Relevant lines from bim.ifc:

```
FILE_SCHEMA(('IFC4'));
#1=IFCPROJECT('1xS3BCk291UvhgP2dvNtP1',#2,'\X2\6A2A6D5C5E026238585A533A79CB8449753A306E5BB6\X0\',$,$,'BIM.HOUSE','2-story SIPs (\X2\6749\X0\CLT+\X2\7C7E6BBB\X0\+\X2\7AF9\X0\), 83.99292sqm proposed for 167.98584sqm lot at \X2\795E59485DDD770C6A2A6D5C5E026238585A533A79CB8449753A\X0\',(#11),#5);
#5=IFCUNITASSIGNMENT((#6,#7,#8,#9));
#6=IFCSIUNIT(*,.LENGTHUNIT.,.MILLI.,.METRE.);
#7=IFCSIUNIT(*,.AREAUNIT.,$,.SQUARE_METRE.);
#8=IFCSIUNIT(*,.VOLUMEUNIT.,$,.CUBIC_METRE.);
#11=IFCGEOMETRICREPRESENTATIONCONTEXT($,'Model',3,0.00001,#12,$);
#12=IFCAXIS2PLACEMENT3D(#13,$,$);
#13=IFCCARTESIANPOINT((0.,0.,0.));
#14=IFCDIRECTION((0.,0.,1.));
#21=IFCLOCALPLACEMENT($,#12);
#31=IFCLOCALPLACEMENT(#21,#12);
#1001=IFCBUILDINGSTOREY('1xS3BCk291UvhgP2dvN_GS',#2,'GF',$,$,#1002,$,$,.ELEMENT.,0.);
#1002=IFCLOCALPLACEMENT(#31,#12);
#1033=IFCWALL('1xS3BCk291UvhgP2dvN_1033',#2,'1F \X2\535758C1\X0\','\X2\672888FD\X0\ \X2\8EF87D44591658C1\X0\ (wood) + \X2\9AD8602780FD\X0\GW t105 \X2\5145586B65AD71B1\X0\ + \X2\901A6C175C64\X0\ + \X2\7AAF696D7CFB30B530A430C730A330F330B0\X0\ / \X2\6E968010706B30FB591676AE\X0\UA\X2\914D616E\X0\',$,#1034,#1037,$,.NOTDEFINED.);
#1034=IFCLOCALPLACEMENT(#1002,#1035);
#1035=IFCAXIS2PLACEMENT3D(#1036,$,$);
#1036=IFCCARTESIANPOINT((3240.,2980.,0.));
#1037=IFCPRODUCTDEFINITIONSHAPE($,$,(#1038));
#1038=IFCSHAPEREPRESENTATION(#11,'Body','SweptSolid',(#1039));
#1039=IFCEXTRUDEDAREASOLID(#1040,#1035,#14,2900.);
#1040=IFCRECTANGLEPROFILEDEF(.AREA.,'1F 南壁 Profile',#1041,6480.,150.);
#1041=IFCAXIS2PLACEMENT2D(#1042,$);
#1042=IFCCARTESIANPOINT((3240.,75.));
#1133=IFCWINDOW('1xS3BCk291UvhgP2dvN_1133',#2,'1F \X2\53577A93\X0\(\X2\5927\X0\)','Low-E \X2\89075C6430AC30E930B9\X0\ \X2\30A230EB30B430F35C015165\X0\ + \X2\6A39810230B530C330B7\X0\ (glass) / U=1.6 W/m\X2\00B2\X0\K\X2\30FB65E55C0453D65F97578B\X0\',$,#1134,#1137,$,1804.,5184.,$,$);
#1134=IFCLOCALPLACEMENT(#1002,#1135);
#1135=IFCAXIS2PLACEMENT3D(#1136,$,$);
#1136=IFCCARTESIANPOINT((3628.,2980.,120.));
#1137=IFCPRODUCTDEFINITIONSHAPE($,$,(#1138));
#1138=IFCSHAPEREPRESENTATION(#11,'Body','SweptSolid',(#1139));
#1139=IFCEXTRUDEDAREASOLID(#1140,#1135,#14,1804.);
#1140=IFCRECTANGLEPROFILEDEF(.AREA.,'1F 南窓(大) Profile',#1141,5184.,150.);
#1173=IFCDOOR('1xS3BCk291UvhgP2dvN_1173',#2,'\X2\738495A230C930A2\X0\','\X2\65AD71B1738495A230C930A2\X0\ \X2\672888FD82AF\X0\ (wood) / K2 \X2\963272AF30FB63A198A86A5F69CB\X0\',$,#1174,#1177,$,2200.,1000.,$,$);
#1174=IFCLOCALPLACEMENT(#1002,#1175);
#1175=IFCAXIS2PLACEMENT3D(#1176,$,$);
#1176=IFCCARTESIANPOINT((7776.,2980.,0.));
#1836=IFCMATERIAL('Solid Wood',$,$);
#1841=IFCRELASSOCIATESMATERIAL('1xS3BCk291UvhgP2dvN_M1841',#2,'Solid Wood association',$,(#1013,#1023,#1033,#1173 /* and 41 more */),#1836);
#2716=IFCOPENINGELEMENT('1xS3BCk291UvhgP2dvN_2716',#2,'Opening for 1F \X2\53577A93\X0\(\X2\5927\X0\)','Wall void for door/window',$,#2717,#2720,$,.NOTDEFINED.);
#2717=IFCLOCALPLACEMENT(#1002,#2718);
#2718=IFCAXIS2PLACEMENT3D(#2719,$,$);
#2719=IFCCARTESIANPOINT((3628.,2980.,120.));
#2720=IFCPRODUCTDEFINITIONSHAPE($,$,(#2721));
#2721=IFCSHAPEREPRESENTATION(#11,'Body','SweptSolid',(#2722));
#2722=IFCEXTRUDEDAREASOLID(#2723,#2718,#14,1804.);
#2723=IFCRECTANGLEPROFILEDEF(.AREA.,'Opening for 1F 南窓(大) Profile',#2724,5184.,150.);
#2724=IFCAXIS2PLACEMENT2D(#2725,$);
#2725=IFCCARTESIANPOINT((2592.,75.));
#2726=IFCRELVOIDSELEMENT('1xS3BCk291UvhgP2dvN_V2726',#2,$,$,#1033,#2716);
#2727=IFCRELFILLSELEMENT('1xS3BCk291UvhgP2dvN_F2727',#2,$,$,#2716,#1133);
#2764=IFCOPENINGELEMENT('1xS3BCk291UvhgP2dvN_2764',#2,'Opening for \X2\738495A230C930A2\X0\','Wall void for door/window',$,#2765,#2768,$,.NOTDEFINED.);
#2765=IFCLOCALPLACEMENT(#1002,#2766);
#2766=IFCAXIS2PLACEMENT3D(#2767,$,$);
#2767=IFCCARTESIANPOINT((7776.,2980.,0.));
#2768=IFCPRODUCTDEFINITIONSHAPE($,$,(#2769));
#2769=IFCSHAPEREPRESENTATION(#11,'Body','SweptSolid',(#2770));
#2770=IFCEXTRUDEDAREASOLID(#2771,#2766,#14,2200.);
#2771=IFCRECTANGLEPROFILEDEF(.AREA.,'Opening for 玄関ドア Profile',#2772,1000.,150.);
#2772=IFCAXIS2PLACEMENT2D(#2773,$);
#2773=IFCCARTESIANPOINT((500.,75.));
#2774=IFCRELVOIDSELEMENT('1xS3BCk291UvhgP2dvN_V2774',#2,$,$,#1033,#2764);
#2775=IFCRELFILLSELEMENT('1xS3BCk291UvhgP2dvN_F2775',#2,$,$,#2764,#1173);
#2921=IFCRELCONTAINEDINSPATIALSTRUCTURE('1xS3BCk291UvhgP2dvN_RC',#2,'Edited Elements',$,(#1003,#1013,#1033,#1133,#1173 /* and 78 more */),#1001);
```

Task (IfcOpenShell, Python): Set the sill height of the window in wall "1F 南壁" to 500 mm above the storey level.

```python
import numpy as np
import ifcopenshell
import ifcopenshell.api.geometry
import ifcopenshell.geom
import ifcopenshell.util.element
import ifcopenshell.util.placement
import ifcopenshell.util.shape
import ifcopenshell.util.unit

model = ifcopenshell.open("bim.ifc")
unit_scale = ifcopenshell.util.unit.calculate_unit_scale(model)

window = model.by_guid("1xS3BCk291UvhgP2dvN_1133")
opening = window.FillsVoids[0].RelatingOpeningElement
storey = ifcopenshell.util.element.get_container(window, ifc_class="IfcBuildingStorey")
level = ifcopenshell.util.placement.get_local_placement(storey.ObjectPlacement)[2, 3]

# The opening's origin need not be at the sill, so measure its lowest point.
shape = ifcopenshell.geom.create_shape(ifcopenshell.geom.settings(), opening)
bottom = ifcopenshell.util.shape.get_shape_bottom_elevation(shape, shape.geometry) / unit_scale
dz = level + 0.5 / unit_scale - bottom

shift = np.array([0.0, 0.0, dz])
# The window is not placed relative to its opening, so move both.
for product in (opening, window):
    matrix = ifcopenshell.util.placement.get_local_placement(product.ObjectPlacement)
    matrix[:3, 3] += shift
    ifcopenshell.api.geometry.edit_object_placement(model, product=product, matrix=matrix, is_si=False)

print(f"moved by {dz * unit_scale:+.3f} m")

model.write("bim_rev.ifc")
```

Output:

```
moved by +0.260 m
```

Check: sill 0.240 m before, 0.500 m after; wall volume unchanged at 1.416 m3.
